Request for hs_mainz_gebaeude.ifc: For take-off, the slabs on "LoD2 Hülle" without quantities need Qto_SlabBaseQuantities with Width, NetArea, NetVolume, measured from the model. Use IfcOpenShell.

First a look at what the model holds.

```python
import ifcopenshell
import ifcopenshell.util.element
import ifcopenshell.util.unit

model = ifcopenshell.open("hs_mainz_gebaeude.ifc")
print(model.schema)
for unit_type in ("LENGTHUNIT", "AREAUNIT", "VOLUMEUNIT"):
    print(unit_type, ifcopenshell.util.unit.calculate_unit_scale(model, unit_type))
storey = next(s for s in model.by_type("IfcBuildingStorey") if s.Name == "LoD2 Hülle")
slabs = [e for e in ifcopenshell.util.element.get_decomposition(storey) if e.is_a("IfcSlab")]
for e in sorted(slabs, key=lambda e: e.id()):
    print(e.id(), e.is_a(), e.Name, list(ifcopenshell.util.element.get_psets(e, qtos_only=True)), sep=" | ")
```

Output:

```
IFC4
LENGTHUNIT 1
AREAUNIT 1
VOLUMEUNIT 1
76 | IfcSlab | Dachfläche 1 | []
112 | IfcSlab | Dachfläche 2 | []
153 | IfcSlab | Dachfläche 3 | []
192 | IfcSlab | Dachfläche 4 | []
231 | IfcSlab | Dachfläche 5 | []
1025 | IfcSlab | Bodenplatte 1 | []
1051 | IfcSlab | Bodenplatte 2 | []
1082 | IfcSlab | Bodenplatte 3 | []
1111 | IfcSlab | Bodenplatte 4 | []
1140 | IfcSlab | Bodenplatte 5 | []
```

```python
import ifcopenshell
import ifcopenshell.api.pset
import ifcopenshell.geom
import ifcopenshell.util.element
import ifcopenshell.util.shape
import ifcopenshell.util.unit

model = ifcopenshell.open("hs_mainz_gebaeude.ifc")
unit_scale = ifcopenshell.util.unit.calculate_unit_scale(model)
area_scale = ifcopenshell.util.unit.calculate_unit_scale(model, "AREAUNIT")
volume_scale = ifcopenshell.util.unit.calculate_unit_scale(model, "VOLUMEUNIT")
settings = ifcopenshell.geom.settings()

storey = next(s for s in model.by_type("IfcBuildingStorey") if s.Name == "LoD2 Hülle")
slabs = [e for e in ifcopenshell.util.element.get_decomposition(storey) if e.is_a("IfcSlab")]

for e in sorted(slabs, key=lambda e: e.id()):
    if ifcopenshell.util.element.get_psets(e, qtos_only=True, should_inherit=False):
        continue
    # Geometry comes back in metres, in the element's own axes.
    shape = ifcopenshell.geom.create_shape(settings, e)
    values = {
        "Width": ifcopenshell.util.shape.get_z(shape.geometry) / unit_scale,
        "NetArea": ifcopenshell.util.shape.get_footprint_area(shape.geometry) / area_scale,
        "NetVolume": ifcopenshell.util.shape.get_volume(shape.geometry) / volume_scale,
    }
    qto = ifcopenshell.api.pset.add_qto(model, product=e, name="Qto_SlabBaseQuantities")
    ifcopenshell.api.pset.edit_qto(model, qto=qto, properties=values)
    print(e.id(), {k: round(v, 3) for k, v in values.items()})

model.write("hs_mainz_gebaeude_rev.ifc")
```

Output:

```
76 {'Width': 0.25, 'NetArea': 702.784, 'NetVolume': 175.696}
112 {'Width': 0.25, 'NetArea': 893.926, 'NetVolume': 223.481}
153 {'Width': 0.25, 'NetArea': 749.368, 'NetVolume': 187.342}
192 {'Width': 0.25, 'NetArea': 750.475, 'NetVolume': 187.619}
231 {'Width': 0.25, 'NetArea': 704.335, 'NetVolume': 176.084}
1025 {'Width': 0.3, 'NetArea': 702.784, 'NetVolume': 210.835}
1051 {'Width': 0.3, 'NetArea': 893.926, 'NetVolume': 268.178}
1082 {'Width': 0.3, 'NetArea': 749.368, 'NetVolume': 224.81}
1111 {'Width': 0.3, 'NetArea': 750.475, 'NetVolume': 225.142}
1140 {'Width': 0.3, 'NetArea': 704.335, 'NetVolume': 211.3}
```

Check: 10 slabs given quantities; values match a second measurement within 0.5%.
